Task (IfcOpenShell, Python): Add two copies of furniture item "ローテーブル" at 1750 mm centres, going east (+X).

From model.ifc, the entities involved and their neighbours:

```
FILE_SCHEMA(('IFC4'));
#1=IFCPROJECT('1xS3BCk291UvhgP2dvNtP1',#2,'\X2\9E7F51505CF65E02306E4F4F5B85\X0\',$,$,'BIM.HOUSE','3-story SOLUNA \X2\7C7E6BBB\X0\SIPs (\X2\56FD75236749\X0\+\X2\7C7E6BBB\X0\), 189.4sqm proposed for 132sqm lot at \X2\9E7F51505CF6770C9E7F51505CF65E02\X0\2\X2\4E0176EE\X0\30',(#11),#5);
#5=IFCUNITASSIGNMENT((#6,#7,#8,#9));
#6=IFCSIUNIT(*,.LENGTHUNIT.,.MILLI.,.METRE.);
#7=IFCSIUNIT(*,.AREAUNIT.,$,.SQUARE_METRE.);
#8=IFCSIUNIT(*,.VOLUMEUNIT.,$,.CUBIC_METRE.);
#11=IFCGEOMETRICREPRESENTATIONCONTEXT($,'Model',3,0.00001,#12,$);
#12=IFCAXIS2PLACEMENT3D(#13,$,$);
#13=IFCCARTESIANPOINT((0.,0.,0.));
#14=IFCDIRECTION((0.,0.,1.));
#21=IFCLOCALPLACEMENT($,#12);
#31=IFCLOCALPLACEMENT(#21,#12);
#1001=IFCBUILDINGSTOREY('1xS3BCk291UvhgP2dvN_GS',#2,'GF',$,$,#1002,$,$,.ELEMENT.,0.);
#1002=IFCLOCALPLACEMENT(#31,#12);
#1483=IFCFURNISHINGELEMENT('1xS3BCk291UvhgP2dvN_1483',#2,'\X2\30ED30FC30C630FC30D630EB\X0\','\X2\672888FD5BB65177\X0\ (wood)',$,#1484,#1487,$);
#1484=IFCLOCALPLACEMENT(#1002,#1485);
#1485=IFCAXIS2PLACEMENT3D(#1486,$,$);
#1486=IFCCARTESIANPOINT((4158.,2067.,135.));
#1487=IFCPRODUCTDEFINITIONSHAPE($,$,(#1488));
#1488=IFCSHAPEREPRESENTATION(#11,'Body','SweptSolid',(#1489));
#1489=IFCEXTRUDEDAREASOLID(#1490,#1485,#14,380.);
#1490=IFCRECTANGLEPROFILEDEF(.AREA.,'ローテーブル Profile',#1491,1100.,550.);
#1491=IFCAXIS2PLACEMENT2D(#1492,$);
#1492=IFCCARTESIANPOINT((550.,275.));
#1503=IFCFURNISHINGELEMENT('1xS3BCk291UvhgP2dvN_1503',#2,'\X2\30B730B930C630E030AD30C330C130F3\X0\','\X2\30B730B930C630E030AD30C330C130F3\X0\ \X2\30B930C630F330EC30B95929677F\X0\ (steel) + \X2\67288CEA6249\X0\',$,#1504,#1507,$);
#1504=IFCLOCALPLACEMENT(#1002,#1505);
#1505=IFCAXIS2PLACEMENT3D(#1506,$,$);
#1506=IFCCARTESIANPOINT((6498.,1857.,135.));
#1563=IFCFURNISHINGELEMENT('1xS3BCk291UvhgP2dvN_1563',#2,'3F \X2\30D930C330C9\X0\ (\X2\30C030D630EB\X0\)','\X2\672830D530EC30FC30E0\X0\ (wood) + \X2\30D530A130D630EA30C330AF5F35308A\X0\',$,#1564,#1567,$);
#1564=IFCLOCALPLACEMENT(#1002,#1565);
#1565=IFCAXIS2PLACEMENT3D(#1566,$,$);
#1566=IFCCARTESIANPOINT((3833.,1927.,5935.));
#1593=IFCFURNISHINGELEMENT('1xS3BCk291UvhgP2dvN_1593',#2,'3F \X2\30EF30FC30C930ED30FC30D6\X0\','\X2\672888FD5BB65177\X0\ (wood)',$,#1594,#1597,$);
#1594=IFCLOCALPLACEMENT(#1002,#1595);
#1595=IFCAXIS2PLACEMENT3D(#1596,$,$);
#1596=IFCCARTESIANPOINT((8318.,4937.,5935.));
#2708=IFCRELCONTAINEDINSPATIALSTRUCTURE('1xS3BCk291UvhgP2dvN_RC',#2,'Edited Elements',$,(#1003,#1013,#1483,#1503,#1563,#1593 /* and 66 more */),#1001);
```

```python
import numpy as np
import ifcopenshell
import ifcopenshell.api.geometry
import ifcopenshell.api.root
import ifcopenshell.util.element
import ifcopenshell.util.placement

model = ifcopenshell.open("model.ifc")


def reuse_history(source, copy):
    """copy_class also copies each property set's owner history, people and application; keep the originals."""
    for rel in copy.IsDefinedBy:
        if rel.is_a("IfcRelDefinesByProperties") and (history := rel.RelatingPropertyDefinition.OwnerHistory):
            rel.RelatingPropertyDefinition.OwnerHistory = source.OwnerHistory
            ifcopenshell.util.element.remove_deep2(model, history)


source = model.by_guid("1xS3BCk291UvhgP2dvN_1483")
base = ifcopenshell.util.placement.get_local_placement(source.ObjectPlacement)
step = np.array([1.0, 0.0, 0.0]) * 1750.0

for i in range(1, 3):
    copy = ifcopenshell.api.root.copy_class(model, product=source)
    copy.Representation = ifcopenshell.util.element.copy_deep(
        model, source.Representation, exclude=["IfcGeometricRepresentationContext", "IfcRepresentationMap"]
    )
    reuse_history(source, copy)
    matrix = base.copy()
    matrix[:3, 3] += i * step
    print("added at", matrix[:3, 3].round(3) + 0.0)
    ifcopenshell.api.geometry.edit_object_placement(model, product=copy, matrix=matrix, is_si=False)

model.write("model-out.ifc")
```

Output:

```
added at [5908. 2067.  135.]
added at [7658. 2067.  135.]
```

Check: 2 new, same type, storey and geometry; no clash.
